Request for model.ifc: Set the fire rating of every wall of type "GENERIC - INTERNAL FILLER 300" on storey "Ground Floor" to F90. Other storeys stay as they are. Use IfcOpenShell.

First a look at what the model holds.

```python
import ifcopenshell
import ifcopenshell.util.element

model = ifcopenshell.open("model.ifc")
print(model.schema)
storey = next(s for s in model.by_type("IfcBuildingStorey") if s.Name == "Ground Floor")
walls = [e for e in ifcopenshell.util.element.get_decomposition(storey) if e.is_a("IfcWall")]
seen = {}
for e in walls:
    element_type = ifcopenshell.util.element.get_type(e)
    key = (element_type.Name if element_type != e and element_type else None, ifcopenshell.util.element.get_pset(e, "Pset_WallCommon", "FireRating"))
    seen[key] = seen.get(key, 0) + 1
for (name, value), count in sorted(seen.items(), key=str):
    print(count, "x", name, "|", value)
```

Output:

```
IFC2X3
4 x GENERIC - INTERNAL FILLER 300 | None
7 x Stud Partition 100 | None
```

```python
import ifcopenshell
import ifcopenshell.api.pset
import ifcopenshell.util.element

model = ifcopenshell.open("model.ifc")

storey = next(s for s in model.by_type("IfcBuildingStorey") if s.Name == "Ground Floor")
walls = [e for e in ifcopenshell.util.element.get_decomposition(storey) if e.is_a("IfcWall")]

count = 0
for e in walls:
    element_type = ifcopenshell.util.element.get_type(e)
    if element_type in (None, e) or element_type.Name != "GENERIC - INTERNAL FILLER 300":
        continue
    # add_pset returns the element's existing set when there is one.
    pset = ifcopenshell.api.pset.add_pset(model, product=e, name="Pset_WallCommon")
    ifcopenshell.api.pset.edit_pset(model, pset=pset, properties={"FireRating": "F90"})
    count += 1

print(count, "walls updated")

model.write("model_updated.ifc")
```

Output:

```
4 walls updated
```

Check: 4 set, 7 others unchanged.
